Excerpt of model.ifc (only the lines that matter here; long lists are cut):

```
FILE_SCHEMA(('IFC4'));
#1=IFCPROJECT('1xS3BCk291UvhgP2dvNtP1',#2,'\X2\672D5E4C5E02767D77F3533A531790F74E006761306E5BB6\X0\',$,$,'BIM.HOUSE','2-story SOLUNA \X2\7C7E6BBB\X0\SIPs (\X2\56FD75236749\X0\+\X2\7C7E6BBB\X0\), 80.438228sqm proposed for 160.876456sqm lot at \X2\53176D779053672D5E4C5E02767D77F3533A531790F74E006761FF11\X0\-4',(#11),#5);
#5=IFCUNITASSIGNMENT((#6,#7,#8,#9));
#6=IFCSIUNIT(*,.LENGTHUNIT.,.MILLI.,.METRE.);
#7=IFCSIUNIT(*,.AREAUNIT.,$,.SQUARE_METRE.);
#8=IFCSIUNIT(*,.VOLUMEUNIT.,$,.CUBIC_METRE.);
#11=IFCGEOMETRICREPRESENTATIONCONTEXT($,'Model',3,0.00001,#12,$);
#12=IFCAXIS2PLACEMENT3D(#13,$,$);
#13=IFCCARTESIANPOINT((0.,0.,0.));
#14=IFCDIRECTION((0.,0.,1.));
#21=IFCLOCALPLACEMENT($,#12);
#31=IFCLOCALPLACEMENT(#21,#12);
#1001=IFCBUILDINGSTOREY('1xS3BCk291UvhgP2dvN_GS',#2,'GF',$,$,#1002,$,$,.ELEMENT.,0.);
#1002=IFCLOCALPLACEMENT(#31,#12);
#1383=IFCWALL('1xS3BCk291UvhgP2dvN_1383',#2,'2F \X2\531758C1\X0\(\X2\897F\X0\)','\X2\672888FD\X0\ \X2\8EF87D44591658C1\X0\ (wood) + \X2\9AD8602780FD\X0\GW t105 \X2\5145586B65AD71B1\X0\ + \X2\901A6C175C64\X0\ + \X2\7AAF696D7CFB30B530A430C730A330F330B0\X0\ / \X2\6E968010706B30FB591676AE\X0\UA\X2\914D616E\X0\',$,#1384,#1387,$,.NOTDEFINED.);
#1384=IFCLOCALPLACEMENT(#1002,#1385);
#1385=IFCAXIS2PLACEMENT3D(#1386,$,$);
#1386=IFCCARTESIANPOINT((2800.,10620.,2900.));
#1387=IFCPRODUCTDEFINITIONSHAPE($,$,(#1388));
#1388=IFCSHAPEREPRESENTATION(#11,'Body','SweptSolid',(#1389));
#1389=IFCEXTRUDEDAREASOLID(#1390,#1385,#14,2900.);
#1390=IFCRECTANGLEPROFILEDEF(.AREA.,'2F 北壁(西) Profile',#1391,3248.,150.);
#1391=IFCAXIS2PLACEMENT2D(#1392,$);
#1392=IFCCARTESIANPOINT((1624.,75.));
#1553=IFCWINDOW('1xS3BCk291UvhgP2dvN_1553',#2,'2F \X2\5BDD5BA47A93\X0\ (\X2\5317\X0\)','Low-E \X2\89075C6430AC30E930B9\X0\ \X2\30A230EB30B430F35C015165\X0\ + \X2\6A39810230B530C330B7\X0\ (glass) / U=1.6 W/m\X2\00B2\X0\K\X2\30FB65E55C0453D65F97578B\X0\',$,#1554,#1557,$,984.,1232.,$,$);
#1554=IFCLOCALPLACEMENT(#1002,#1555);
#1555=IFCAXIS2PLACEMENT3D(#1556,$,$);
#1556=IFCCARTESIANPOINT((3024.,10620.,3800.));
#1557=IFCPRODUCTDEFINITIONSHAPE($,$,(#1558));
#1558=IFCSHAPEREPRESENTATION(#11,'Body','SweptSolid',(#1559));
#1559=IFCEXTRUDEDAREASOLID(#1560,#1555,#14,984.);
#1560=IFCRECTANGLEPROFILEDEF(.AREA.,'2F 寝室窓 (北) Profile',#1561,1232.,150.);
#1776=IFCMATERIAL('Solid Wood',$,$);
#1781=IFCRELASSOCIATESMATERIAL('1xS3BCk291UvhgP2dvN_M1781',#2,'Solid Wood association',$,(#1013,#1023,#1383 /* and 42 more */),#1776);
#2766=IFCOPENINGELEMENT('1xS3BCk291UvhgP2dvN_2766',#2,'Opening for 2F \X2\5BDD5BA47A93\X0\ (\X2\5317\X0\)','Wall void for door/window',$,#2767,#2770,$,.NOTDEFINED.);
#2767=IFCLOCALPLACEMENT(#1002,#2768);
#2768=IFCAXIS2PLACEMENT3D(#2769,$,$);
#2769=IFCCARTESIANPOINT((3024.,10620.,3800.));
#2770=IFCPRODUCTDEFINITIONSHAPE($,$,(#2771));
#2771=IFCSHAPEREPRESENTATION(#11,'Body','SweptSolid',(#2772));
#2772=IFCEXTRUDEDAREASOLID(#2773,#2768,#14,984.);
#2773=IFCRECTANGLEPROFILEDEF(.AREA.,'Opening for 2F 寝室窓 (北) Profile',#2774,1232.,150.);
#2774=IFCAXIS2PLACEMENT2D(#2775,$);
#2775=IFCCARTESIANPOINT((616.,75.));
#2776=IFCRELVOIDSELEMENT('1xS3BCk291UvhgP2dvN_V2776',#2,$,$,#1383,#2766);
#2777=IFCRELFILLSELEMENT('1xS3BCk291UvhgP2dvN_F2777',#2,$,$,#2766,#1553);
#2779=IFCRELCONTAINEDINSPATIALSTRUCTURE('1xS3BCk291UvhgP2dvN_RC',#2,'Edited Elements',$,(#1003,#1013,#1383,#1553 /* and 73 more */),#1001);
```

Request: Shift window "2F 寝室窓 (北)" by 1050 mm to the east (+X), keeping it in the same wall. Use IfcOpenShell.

```python
import ifcopenshell
import ifcopenshell.api.geometry
import ifcopenshell.util.placement
import ifcopenshell.util.unit

model = ifcopenshell.open("model.ifc")
unit_scale = ifcopenshell.util.unit.calculate_unit_scale(model)

window = model.by_guid("1xS3BCk291UvhgP2dvN_1553")
opening = window.FillsVoids[0].RelatingOpeningElement
wall = opening.VoidsElements[0].RelatingBuildingElement

wall_matrix = ifcopenshell.util.placement.get_local_placement(wall.ObjectPlacement)
shift = wall_matrix[:3, 0] * 1.05 / unit_scale
before = ifcopenshell.util.placement.get_local_placement(window.ObjectPlacement)[:3, 3].copy()

# The window is not placed relative to its opening, so move both.
for product in (opening, window):
    matrix = ifcopenshell.util.placement.get_local_placement(product.ObjectPlacement)
    matrix[:3, 3] += shift
    ifcopenshell.api.geometry.edit_object_placement(model, product=product, matrix=matrix, is_si=False)

after = ifcopenshell.util.placement.get_local_placement(window.ObjectPlacement)[:3, 3]
print("window moved by", (after - before).round(3) + 0.0)

model.write("model_edited.ifc")
```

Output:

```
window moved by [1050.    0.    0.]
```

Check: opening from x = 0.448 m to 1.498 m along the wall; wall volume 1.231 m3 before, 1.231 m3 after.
